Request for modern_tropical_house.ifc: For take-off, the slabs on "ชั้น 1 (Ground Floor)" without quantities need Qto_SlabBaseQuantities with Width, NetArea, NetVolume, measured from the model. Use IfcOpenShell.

First a look at what the model holds.

```python
import ifcopenshell
import ifcopenshell.util.element
import ifcopenshell.util.unit

model = ifcopenshell.open("modern_tropical_house.ifc")
print(model.schema)
for unit_type in ("LENGTHUNIT", "AREAUNIT", "VOLUMEUNIT"):
    print(unit_type, ifcopenshell.util.unit.calculate_unit_scale(model, unit_type))
storey = next(s for s in model.by_type("IfcBuildingStorey") if s.Name == "ชั้น 1 (Ground Floor)")
slabs = [e for e in ifcopenshell.util.element.get_decomposition(storey) if e.is_a("IfcSlab")]
for e in sorted(slabs, key=lambda e: e.id()):
    print(e.id(), e.is_a(), e.Name, list(ifcopenshell.util.element.get_psets(e, qtos_only=True)), sep=" | ")
```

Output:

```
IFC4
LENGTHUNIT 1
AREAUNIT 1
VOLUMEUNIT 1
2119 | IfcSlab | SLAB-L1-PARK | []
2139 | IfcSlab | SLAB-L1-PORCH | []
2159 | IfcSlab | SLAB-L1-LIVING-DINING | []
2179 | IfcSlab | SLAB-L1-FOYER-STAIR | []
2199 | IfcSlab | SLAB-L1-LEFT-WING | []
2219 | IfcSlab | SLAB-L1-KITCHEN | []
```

```python
import ifcopenshell
import ifcopenshell.api.pset
import ifcopenshell.geom
import ifcopenshell.util.element
import ifcopenshell.util.shape
import ifcopenshell.util.unit

model = ifcopenshell.open("modern_tropical_house.ifc")
unit_scale = ifcopenshell.util.unit.calculate_unit_scale(model)
area_scale = ifcopenshell.util.unit.calculate_unit_scale(model, "AREAUNIT")
volume_scale = ifcopenshell.util.unit.calculate_unit_scale(model, "VOLUMEUNIT")
settings = ifcopenshell.geom.settings()

storey = next(s for s in model.by_type("IfcBuildingStorey") if s.Name == "ชั้น 1 (Ground Floor)")
slabs = [e for e in ifcopenshell.util.element.get_decomposition(storey) if e.is_a("IfcSlab")]

for e in sorted(slabs, key=lambda e: e.id()):
    if ifcopenshell.util.element.get_psets(e, qtos_only=True, should_inherit=False):
        continue
    # Geometry comes back in metres, in the element's own axes.
    shape = ifcopenshell.geom.create_shape(settings, e)
    values = {
        "Width": ifcopenshell.util.shape.get_z(shape.geometry) / unit_scale,
        "NetArea": ifcopenshell.util.shape.get_footprint_area(shape.geometry) / area_scale,
        "NetVolume": ifcopenshell.util.shape.get_volume(shape.geometry) / volume_scale,
    }
    qto = ifcopenshell.api.pset.add_qto(model, product=e, name="Qto_SlabBaseQuantities")
    ifcopenshell.api.pset.edit_qto(model, qto=qto, properties=values)
    print(e.id(), {k: round(v, 3) for k, v in values.items()})

model.write("modern_tropical_house_updated.ifc")
```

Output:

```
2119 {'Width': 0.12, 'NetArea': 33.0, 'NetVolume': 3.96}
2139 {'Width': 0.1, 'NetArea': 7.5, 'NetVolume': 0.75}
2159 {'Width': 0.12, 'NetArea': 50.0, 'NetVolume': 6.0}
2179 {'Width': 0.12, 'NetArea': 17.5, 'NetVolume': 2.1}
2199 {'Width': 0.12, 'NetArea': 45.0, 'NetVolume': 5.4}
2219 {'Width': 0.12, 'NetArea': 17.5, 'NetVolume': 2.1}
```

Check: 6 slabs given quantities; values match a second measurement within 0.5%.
